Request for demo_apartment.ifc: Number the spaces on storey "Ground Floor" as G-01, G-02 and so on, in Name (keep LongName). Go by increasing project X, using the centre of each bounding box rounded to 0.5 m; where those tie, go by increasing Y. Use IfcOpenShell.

First a look at what the model holds.

```python
import ifcopenshell
import ifcopenshell.util.element
import ifcopenshell.util.placement

model = ifcopenshell.open("demo_apartment.ifc")
print(model.schema)
storey = next(s for s in model.by_type("IfcBuildingStorey") if s.Name == "Ground Floor")
spaces = [e for e in ifcopenshell.util.element.get_decomposition(storey) if e.is_a("IfcSpace")]
for e in sorted(spaces, key=lambda e: e.id()):
    origin = ifcopenshell.util.placement.get_local_placement(e.ObjectPlacement)[:3, 3]
    print(e.id(), e.Name, e.LongName, origin.round(2) + 0.0, sep=" | ")
```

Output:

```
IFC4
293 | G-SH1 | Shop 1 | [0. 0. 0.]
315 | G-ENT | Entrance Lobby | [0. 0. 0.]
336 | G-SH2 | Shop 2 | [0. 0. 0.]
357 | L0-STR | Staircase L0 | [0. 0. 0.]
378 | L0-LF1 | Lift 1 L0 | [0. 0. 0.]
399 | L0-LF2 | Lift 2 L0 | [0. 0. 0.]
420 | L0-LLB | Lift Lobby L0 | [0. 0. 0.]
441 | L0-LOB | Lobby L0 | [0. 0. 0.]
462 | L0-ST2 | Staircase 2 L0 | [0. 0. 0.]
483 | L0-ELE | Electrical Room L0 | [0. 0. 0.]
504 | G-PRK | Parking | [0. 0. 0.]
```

```python
import ifcopenshell
import ifcopenshell.geom
import ifcopenshell.util.element
import ifcopenshell.util.shape

model = ifcopenshell.open("demo_apartment.ifc")
settings = ifcopenshell.geom.settings()
settings.set("use-world-coords", True)


def centre(element):
    shape = ifcopenshell.geom.create_shape(settings, element)
    return ifcopenshell.util.shape.get_bbox_centroid(shape.geometry)


storey = next(s for s in model.by_type("IfcBuildingStorey") if s.Name == "Ground Floor")
spaces = [e for e in ifcopenshell.util.element.get_decomposition(storey) if e.is_a("IfcSpace")]

# Insertion points can sit at a corner or the storey origin, so sort by the geometry (in metres).
centres = {e: centre(e) for e in spaces}
spaces.sort(key=lambda e: (round(centres[e][0] / 0.5), centres[e][1]))

for i, e in enumerate(spaces, start=1):
    number = f"G-{i:02d}"
    e.Name = number
    print(e.id(), number)

model.write("demo_apartment-out.ifc")
```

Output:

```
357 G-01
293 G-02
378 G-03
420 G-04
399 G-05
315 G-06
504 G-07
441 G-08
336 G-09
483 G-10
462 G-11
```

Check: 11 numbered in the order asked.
